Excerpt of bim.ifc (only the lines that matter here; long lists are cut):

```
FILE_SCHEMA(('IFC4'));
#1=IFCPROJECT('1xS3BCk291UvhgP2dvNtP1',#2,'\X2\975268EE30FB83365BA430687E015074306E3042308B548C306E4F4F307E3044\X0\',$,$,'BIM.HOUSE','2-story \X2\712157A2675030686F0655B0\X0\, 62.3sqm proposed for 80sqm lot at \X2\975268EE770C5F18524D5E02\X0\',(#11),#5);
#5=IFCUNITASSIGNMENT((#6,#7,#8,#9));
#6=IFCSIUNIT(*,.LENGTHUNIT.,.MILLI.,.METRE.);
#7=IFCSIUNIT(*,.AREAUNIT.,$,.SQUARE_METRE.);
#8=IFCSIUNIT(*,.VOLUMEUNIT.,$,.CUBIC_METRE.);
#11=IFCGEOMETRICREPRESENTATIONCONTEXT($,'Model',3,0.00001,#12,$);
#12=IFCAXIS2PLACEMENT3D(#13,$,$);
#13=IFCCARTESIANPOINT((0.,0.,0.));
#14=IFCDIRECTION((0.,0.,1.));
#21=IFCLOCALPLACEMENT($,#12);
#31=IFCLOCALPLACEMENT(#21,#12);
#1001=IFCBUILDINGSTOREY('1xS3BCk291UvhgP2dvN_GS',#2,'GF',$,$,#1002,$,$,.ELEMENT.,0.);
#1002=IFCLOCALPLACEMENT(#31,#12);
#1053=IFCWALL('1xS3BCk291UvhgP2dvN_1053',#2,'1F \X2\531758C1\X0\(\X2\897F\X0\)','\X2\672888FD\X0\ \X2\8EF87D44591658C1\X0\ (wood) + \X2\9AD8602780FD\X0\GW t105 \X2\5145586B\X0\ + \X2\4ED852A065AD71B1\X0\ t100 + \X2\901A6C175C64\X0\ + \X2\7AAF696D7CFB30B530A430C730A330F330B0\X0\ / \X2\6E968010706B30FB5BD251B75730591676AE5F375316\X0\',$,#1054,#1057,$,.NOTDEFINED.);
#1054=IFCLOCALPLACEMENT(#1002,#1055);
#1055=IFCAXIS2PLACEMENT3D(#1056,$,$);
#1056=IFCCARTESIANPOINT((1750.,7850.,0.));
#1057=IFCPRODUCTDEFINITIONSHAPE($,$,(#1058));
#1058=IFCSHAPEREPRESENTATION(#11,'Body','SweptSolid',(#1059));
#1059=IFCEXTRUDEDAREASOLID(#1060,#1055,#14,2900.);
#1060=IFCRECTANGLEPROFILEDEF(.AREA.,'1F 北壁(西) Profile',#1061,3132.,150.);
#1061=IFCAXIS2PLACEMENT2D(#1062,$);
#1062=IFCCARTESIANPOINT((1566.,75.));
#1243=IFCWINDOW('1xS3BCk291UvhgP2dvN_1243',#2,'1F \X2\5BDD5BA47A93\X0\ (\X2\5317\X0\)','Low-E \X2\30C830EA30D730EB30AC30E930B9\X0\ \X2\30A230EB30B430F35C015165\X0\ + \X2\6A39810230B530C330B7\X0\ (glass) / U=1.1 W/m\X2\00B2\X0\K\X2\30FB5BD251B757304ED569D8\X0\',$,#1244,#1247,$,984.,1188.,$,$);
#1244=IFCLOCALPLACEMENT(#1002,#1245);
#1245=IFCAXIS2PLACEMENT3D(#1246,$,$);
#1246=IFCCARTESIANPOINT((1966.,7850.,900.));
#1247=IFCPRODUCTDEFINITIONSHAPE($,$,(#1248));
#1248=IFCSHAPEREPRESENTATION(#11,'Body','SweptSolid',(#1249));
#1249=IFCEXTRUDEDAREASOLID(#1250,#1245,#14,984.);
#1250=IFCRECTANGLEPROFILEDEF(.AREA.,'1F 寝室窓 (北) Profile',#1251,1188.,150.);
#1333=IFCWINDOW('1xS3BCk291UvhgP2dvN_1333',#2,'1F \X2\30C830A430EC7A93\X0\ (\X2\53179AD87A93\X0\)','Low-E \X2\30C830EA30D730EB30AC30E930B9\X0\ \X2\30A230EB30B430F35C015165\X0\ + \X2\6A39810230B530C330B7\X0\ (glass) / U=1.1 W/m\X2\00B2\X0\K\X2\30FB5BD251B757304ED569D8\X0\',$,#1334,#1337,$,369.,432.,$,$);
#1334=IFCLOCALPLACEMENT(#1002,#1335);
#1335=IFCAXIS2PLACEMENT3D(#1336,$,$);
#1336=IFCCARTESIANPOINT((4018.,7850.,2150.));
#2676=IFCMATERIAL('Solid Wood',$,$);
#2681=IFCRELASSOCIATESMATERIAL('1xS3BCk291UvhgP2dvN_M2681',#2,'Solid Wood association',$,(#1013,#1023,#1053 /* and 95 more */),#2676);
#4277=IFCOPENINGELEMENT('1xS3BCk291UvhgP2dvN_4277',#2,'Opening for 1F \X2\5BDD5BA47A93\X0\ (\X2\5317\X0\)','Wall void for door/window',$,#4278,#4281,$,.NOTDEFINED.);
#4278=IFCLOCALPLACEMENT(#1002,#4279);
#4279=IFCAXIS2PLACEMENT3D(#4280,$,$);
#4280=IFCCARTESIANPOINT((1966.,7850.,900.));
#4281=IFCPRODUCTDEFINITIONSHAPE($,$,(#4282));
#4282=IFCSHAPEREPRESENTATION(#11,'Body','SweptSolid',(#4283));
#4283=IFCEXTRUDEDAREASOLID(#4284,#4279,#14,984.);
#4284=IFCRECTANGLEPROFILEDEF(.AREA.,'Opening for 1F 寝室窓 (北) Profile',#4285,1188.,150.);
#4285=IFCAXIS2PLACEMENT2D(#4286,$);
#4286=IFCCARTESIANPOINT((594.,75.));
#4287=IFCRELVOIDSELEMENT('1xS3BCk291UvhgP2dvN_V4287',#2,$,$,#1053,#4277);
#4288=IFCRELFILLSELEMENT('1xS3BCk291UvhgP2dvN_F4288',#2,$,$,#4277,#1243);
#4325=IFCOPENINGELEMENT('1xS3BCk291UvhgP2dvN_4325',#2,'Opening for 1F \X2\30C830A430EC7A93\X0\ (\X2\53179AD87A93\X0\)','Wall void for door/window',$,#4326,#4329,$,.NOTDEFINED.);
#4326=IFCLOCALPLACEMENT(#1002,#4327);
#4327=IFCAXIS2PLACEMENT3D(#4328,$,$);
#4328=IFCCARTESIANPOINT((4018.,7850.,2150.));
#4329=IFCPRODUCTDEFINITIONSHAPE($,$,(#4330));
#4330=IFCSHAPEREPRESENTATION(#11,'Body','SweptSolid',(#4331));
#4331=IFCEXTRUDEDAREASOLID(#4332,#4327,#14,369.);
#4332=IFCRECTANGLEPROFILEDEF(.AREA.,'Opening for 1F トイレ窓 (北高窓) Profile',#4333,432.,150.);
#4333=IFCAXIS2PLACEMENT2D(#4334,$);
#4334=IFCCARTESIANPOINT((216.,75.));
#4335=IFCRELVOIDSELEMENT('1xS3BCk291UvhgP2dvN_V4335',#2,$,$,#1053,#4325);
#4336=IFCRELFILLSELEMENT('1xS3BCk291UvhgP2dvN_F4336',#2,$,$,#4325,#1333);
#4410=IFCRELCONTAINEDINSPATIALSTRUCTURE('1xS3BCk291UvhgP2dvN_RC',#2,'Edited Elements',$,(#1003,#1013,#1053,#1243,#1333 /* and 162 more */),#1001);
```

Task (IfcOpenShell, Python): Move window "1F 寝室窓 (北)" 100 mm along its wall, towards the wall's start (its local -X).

```python
import ifcopenshell
import ifcopenshell.api.geometry
import ifcopenshell.util.placement
import ifcopenshell.util.unit

model = ifcopenshell.open("bim.ifc")
unit_scale = ifcopenshell.util.unit.calculate_unit_scale(model)

window = model.by_guid("1xS3BCk291UvhgP2dvN_1243")
opening = window.FillsVoids[0].RelatingOpeningElement
wall = opening.VoidsElements[0].RelatingBuildingElement

wall_matrix = ifcopenshell.util.placement.get_local_placement(wall.ObjectPlacement)
shift = wall_matrix[:3, 0] * -0.1 / unit_scale
before = ifcopenshell.util.placement.get_local_placement(window.ObjectPlacement)[:3, 3].copy()

# The window is not placed relative to its opening, so move both.
for product in (opening, window):
    matrix = ifcopenshell.util.placement.get_local_placement(product.ObjectPlacement)
    matrix[:3, 3] += shift
    ifcopenshell.api.geometry.edit_object_placement(model, product=product, matrix=matrix, is_si=False)

after = ifcopenshell.util.placement.get_local_placement(window.ObjectPlacement)[:3, 3]
print("window moved by", (after - before).round(3) + 0.0)

model.write("bim_v2.ifc")
```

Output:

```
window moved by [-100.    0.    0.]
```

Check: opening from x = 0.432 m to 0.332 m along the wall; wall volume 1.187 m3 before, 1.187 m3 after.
